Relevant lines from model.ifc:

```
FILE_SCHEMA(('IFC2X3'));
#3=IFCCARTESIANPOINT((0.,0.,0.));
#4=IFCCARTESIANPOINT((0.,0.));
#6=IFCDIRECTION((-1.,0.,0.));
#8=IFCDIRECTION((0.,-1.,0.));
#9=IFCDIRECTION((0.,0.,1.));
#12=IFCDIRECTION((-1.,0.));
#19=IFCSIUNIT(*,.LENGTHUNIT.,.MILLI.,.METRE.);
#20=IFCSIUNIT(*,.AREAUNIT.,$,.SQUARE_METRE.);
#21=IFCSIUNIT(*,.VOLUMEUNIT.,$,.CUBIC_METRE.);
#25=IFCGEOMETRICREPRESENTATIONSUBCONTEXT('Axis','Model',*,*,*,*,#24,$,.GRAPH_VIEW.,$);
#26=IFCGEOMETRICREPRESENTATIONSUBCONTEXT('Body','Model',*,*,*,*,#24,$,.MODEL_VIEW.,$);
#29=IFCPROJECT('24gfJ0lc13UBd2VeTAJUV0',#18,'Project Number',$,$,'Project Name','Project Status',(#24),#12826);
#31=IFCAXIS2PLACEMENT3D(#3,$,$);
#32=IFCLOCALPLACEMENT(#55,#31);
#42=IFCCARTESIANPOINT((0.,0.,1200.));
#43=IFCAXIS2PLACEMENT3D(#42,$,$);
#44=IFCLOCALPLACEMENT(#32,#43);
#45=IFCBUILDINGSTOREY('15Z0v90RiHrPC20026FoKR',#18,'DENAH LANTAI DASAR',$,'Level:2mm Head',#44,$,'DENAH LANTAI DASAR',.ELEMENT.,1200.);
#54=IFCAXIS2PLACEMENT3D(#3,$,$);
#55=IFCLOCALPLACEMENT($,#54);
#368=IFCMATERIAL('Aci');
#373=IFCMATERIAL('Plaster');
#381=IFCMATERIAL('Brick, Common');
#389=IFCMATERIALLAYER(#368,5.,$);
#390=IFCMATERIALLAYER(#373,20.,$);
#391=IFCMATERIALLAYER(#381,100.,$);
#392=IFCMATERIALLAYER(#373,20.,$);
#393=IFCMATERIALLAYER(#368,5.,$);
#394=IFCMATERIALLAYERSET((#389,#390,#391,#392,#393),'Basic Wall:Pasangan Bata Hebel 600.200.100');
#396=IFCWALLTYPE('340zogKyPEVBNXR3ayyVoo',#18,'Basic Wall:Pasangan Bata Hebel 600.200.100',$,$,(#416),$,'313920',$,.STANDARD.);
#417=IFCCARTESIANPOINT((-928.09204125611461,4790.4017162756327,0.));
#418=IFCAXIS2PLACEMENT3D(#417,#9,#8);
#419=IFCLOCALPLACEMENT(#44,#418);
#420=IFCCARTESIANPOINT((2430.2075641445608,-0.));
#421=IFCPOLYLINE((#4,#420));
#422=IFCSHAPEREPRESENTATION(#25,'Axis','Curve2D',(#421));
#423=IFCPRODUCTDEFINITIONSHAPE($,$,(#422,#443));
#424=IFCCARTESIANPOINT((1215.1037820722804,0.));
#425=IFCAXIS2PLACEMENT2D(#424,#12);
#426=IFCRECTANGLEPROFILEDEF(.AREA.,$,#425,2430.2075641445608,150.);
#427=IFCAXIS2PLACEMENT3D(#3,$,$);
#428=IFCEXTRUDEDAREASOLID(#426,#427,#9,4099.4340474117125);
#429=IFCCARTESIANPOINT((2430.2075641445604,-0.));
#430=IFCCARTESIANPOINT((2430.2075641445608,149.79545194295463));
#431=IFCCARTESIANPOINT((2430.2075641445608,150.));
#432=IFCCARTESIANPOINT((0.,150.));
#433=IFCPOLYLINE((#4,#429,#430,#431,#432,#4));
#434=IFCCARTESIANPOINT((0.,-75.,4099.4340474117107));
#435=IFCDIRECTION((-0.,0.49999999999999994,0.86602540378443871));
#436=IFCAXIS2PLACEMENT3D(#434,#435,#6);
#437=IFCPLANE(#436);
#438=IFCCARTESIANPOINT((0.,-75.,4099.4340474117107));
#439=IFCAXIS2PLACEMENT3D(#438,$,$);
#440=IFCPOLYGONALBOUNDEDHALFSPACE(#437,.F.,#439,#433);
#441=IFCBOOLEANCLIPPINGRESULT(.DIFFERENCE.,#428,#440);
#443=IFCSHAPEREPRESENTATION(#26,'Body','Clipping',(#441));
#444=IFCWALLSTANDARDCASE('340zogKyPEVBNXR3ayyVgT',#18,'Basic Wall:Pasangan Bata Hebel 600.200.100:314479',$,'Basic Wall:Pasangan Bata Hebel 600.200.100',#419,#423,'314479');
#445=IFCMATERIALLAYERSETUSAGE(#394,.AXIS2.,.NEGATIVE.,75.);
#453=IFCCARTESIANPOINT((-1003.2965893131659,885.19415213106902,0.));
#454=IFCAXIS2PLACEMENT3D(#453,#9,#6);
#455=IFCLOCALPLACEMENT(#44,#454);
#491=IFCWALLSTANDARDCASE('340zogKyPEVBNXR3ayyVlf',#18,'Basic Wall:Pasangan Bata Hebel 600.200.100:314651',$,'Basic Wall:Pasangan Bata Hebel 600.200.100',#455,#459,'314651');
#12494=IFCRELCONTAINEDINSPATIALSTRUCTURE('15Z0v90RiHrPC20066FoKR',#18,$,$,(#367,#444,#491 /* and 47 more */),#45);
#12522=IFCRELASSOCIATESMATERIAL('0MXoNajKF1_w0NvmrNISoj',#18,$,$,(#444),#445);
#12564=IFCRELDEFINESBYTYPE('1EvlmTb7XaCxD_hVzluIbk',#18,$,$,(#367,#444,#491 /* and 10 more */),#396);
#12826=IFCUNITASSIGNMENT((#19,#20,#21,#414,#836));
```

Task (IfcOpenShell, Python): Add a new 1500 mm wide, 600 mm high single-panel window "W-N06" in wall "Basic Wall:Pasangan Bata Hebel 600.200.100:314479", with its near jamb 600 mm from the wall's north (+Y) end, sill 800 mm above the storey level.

```python
import numpy as np
import ifcopenshell
import ifcopenshell.api.feature
import ifcopenshell.api.geometry
import ifcopenshell.api.root
import ifcopenshell.api.spatial
import ifcopenshell.api.type
import ifcopenshell.geom
import ifcopenshell.util.element
import ifcopenshell.util.placement
import ifcopenshell.util.representation
import ifcopenshell.util.shape
import ifcopenshell.util.unit

model = ifcopenshell.open("model.ifc")
unit_scale = ifcopenshell.util.unit.calculate_unit_scale(model)
settings = ifcopenshell.geom.settings()


def volume(element):
    """Net volume in cubic metres, openings subtracted."""
    shape = ifcopenshell.geom.create_shape(settings, element)
    return ifcopenshell.util.shape.get_volume(shape.geometry)


wall = model.by_guid("340zogKyPEVBNXR3ayyVgT")
storey = ifcopenshell.util.element.get_container(wall, ifc_class="IfcBuildingStorey")
context = ifcopenshell.util.representation.get_context(model, "Model", "Body", "MODEL_VIEW")
before = volume(wall)

width, height, from_end, sill = 1.5, 0.6, 0.6, 0.8  # metres

# The wall runs along its own X axis, and the end named is its -X end.
wall_shape = ifcopenshell.geom.create_shape(settings, wall)
x, y, z = ifcopenshell.util.shape.get_vertices(wall_shape.geometry).T
start = x.min() + from_end
face, thickness = float(y.min()), float(y.max() - y.min())
wall_matrix = ifcopenshell.util.placement.get_local_placement(wall.ObjectPlacement)
level = ifcopenshell.util.placement.get_local_placement(storey.ObjectPlacement)[2, 3]


def in_wall(x, y):
    """Placement at x, y metres in the wall's axes, at sill height."""
    matrix = wall_matrix.copy()
    matrix[:, 3] = wall_matrix @ np.array([x / unit_scale, y / unit_scale, 0.0, 1.0])
    matrix[2, 3] = level + sill / unit_scale
    return matrix


# Opening: a box that overshoots both wall faces by 50 mm.
opening = ifcopenshell.api.root.create_entity(model, ifc_class="IfcOpeningElement")
box = ifcopenshell.api.geometry.add_wall_representation(
    model, context=context, length=width, height=height, thickness=thickness + 0.1
)
ifcopenshell.api.geometry.assign_representation(model, product=opening, representation=box)
ifcopenshell.api.geometry.edit_object_placement(model, product=opening, matrix=in_wall(start, face - 0.05), is_si=False)
ifcopenshell.api.feature.add_feature(model, feature=opening, element=wall)

window = ifcopenshell.api.root.create_entity(model, ifc_class="IfcWindow", name="W-N06")
window.OverallWidth, window.OverallHeight = width / unit_scale, height / unit_scale
body = ifcopenshell.api.geometry.add_window_representation(
    model,
    context=context,
    overall_width=window.OverallWidth,
    overall_height=window.OverallHeight,
    partition_type="SINGLE_PANEL",
)
ifcopenshell.api.geometry.assign_representation(model, product=window, representation=body)
ifcopenshell.api.spatial.assign_container(model, products=[window], relating_structure=storey)
fills = ifcopenshell.api.feature.add_filling(model, opening=opening, element=window)
fills.OwnerHistory = window.OwnerHistory  # required in IFC2X3

# IFC2X3 keeps the operation on the window style.
style = ifcopenshell.api.root.create_entity(model, ifc_class="IfcWindowStyle", name="W-N06")
style.OperationType, style.ConstructionType = "SINGLE_PANEL", "NOTDEFINED"
style.ParameterTakesPrecedence = style.Sizeable = False
ifcopenshell.api.type.assign_type(model, related_objects=[window], relating_type=style)

# Centre the window in the wall's thickness.
ifcopenshell.api.geometry.edit_object_placement(model, product=window, matrix=in_wall(start, face), is_si=False)
window_shape = ifcopenshell.geom.create_shape(settings, window)
depth = ifcopenshell.util.shape.get_vertices(window_shape.geometry)[:, 1]
offset = face + thickness / 2 - (depth.min() + depth.max()) / 2
ifcopenshell.api.geometry.edit_object_placement(model, product=window, matrix=in_wall(start, offset), is_si=False)

after = volume(wall)

print(f"wall volume {before:.3f} -> {after:.3f} m3")

model.write("model_v2.ifc")
```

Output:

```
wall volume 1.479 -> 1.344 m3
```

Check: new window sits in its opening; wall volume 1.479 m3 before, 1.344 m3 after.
